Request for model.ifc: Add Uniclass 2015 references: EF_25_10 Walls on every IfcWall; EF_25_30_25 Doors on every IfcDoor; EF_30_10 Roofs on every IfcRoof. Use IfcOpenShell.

First a look at what the model holds.

```python
import ifcopenshell

model = ifcopenshell.open("model.ifc")
print(model.schema)
print("classifications:", [c.Name for c in model.by_type("IfcClassification")])
for ifc_class in ("IfcDoor", "IfcRoof", "IfcStair", "IfcWall", "IfcWindow"):
    print(ifc_class, len(model.by_type(ifc_class)))
```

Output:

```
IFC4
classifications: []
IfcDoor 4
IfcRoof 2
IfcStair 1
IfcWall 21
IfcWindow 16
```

```python
import ifcopenshell
import ifcopenshell.api.classification

model = ifcopenshell.open("model.ifc")

system = ifcopenshell.api.classification.add_classification(model, classification="Uniclass 2015")

codes = {
    "IfcWall": ("EF_25_10", "Walls"),
    "IfcDoor": ("EF_25_30_25", "Doors"),
    "IfcRoof": ("EF_30_10", "Roofs"),
}
for ifc_class, (code, name) in codes.items():
    products = model.by_type(ifc_class)
    ifcopenshell.api.classification.add_reference(
        model, products=products, classification=system, identification=code, name=name
    )
    print(code, len(products))

model.write("model-out.ifc")
```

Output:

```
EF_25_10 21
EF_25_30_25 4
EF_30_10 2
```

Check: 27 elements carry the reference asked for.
